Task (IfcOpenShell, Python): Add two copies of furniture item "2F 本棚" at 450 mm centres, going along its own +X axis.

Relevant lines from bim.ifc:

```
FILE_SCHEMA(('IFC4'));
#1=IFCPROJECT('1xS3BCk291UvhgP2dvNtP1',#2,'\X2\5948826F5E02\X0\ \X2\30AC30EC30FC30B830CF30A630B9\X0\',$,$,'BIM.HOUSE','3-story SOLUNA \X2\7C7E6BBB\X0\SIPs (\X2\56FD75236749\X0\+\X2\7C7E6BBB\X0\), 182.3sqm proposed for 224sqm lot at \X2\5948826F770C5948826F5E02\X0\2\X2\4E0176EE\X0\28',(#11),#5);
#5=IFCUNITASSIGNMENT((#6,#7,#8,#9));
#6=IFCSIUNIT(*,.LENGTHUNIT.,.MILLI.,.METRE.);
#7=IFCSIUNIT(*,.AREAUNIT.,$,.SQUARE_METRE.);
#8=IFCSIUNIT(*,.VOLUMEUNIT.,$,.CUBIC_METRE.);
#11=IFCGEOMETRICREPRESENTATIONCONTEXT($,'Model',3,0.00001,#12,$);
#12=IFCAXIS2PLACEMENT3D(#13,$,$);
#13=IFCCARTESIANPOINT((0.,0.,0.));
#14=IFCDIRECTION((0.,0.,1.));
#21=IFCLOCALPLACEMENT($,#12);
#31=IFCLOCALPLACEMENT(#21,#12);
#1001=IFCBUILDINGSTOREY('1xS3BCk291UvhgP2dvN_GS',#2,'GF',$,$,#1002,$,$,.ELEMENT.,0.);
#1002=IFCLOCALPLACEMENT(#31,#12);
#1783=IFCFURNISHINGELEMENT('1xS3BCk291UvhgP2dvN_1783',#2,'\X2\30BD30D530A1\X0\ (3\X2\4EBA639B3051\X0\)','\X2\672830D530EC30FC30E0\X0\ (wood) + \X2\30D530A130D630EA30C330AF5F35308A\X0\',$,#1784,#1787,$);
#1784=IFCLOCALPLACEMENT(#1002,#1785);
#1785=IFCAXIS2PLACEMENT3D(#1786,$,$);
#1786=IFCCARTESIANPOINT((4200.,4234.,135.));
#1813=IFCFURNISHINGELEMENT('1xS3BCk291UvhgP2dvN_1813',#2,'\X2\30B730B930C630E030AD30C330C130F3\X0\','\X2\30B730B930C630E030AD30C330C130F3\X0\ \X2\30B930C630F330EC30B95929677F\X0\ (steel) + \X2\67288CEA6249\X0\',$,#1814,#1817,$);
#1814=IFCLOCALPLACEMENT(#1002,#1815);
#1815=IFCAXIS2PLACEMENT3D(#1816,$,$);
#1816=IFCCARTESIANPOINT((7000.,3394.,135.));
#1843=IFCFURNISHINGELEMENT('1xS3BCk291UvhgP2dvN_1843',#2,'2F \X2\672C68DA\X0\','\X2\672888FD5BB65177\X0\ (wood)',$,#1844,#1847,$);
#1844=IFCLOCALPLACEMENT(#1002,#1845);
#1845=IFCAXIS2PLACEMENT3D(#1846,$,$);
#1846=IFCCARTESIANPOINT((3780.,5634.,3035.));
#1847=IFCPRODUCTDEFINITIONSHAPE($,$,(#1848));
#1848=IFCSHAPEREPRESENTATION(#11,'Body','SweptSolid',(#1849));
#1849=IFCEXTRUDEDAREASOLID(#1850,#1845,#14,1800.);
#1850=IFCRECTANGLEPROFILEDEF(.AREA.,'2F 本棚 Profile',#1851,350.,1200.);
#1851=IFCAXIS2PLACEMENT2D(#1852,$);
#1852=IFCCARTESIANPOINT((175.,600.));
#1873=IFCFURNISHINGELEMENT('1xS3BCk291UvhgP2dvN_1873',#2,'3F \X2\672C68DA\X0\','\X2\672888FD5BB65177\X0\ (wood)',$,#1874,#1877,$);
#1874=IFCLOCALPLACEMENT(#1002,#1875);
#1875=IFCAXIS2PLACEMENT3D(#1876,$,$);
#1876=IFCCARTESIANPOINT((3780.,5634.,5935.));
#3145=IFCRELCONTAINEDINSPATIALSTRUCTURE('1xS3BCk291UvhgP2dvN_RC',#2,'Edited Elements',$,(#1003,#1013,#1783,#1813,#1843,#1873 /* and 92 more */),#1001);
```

```python
import ifcopenshell
import ifcopenshell.api.geometry
import ifcopenshell.api.root
import ifcopenshell.util.element
import ifcopenshell.util.placement

model = ifcopenshell.open("bim.ifc")


def reuse_history(source, copy):
    """copy_class also copies each property set's owner history, people and application; keep the originals."""
    for rel in copy.IsDefinedBy:
        if rel.is_a("IfcRelDefinesByProperties") and (history := rel.RelatingPropertyDefinition.OwnerHistory):
            rel.RelatingPropertyDefinition.OwnerHistory = source.OwnerHistory
            ifcopenshell.util.element.remove_deep2(model, history)


source = model.by_guid("1xS3BCk291UvhgP2dvN_1843")
base = ifcopenshell.util.placement.get_local_placement(source.ObjectPlacement)
step = base[:3, 0] * 450.0

for i in range(1, 3):
    copy = ifcopenshell.api.root.copy_class(model, product=source)
    copy.Representation = ifcopenshell.util.element.copy_deep(
        model, source.Representation, exclude=["IfcGeometricRepresentationContext", "IfcRepresentationMap"]
    )
    reuse_history(source, copy)
    matrix = base.copy()
    matrix[:3, 3] += i * step
    print("added at", matrix[:3, 3].round(3) + 0.0)
    ifcopenshell.api.geometry.edit_object_placement(model, product=copy, matrix=matrix, is_si=False)

model.write("bim-out.ifc")
```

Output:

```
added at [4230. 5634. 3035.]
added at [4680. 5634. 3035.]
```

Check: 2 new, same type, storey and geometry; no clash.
